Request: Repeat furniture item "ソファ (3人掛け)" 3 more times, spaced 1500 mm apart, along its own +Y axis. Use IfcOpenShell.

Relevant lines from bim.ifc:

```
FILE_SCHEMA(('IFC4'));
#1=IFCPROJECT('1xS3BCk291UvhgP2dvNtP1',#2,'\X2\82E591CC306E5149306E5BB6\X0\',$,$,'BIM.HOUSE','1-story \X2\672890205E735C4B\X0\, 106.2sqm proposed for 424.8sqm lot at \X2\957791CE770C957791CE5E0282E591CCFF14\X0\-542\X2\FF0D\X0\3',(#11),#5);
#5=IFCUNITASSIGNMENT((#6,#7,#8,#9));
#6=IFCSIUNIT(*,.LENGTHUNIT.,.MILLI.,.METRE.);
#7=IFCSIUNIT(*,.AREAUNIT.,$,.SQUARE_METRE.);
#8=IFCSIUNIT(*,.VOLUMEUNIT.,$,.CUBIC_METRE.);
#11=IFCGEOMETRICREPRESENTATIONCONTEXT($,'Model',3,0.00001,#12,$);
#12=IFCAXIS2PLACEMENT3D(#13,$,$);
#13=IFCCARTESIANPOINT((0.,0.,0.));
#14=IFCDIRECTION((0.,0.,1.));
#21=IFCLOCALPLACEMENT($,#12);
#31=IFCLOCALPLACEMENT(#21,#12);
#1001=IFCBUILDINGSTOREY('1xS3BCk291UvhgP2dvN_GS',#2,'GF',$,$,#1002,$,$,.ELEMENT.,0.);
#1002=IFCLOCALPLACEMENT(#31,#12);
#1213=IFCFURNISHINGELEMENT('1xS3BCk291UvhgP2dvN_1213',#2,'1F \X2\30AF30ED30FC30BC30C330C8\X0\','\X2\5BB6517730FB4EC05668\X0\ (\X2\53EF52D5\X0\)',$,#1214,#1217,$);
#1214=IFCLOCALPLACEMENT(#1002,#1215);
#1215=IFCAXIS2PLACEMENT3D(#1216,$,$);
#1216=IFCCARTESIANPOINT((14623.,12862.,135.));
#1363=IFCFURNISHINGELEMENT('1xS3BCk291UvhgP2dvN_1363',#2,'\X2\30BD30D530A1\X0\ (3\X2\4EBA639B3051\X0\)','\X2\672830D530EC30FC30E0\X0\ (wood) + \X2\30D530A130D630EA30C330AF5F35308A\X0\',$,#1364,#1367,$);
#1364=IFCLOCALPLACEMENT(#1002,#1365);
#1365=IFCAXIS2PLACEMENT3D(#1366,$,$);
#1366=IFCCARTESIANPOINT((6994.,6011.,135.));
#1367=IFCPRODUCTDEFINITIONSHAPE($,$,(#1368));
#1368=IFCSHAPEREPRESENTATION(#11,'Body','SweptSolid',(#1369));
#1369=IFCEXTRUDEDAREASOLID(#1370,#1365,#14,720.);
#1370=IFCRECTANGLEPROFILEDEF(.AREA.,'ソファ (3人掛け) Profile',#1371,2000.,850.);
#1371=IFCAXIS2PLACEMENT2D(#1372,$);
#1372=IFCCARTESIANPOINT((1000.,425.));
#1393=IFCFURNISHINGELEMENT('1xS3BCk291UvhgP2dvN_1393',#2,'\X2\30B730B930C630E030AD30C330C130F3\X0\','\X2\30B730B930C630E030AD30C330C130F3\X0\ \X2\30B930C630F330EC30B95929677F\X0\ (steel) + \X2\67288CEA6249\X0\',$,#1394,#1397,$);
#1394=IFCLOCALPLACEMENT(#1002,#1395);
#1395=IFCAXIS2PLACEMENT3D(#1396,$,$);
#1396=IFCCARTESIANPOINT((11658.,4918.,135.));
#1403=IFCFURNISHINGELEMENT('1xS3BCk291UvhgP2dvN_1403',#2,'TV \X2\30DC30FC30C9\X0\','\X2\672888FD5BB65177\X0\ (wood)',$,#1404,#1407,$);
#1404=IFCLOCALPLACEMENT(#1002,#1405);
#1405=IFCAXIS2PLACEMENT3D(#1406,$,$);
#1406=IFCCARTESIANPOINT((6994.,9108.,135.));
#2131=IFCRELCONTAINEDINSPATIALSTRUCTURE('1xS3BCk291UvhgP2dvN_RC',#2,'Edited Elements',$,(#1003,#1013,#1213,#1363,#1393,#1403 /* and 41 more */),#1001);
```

```python
import ifcopenshell
import ifcopenshell.api.geometry
import ifcopenshell.api.root
import ifcopenshell.util.element
import ifcopenshell.util.placement
import ifcopenshell.util.unit

model = ifcopenshell.open("bim.ifc")
unit_scale = ifcopenshell.util.unit.calculate_unit_scale(model)


def reuse_history(source, copy):
    """copy_class also copies each property set's owner history, people and application; keep the originals."""
    for rel in copy.IsDefinedBy:
        if rel.is_a("IfcRelDefinesByProperties") and (history := rel.RelatingPropertyDefinition.OwnerHistory):
            rel.RelatingPropertyDefinition.OwnerHistory = source.OwnerHistory
            ifcopenshell.util.element.remove_deep2(model, history)


source = model.by_id(1363)
base = ifcopenshell.util.placement.get_local_placement(source.ObjectPlacement)
step = base[:3, 1] * 1.5 / unit_scale

for i in range(1, 4):
    copy = ifcopenshell.api.root.copy_class(model, product=source)
    copy.Representation = ifcopenshell.util.element.copy_deep(
        model, source.Representation, exclude=["IfcGeometricRepresentationContext", "IfcRepresentationMap"]
    )
    reuse_history(source, copy)
    matrix = base.copy()
    matrix[:3, 3] += i * step
    print("added at", matrix[:3, 3].round(3) + 0.0)
    ifcopenshell.api.geometry.edit_object_placement(model, product=copy, matrix=matrix, is_si=False)

model.write("bim_edited.ifc")
```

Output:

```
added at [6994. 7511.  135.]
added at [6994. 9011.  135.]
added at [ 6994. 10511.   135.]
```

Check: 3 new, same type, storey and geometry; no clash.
